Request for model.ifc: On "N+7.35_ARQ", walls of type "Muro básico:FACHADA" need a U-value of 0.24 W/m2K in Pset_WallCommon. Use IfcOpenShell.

First a look at what the model holds.

```python
import ifcopenshell
import ifcopenshell.util.element

model = ifcopenshell.open("model.ifc")
print(model.schema)
storey = next(s for s in model.by_type("IfcBuildingStorey") if s.Name == "N+7.35_ARQ")
walls = [e for e in ifcopenshell.util.element.get_decomposition(storey) if e.is_a("IfcWall")]
seen = {}
for e in walls:
    element_type = ifcopenshell.util.element.get_type(e)
    key = (element_type.Name if element_type != e and element_type else None, ifcopenshell.util.element.get_pset(e, "Pset_WallCommon", "ThermalTransmittance"))
    seen[key] = seen.get(key, 0) + 1
for (name, value), count in sorted(seen.items(), key=str):
    print(count, "x", name, "|", value)
```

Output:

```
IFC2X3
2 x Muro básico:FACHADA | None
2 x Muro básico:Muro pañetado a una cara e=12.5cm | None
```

```python
import ifcopenshell
import ifcopenshell.api.pset
import ifcopenshell.util.element

model = ifcopenshell.open("model.ifc")

storey = next(s for s in model.by_type("IfcBuildingStorey") if s.Name == "N+7.35_ARQ")
walls = [e for e in ifcopenshell.util.element.get_decomposition(storey) if e.is_a("IfcWall")]

count = 0
for e in walls:
    element_type = ifcopenshell.util.element.get_type(e)
    if element_type in (None, e) or element_type.Name != "Muro básico:FACHADA":
        continue
    # add_pset returns the element's existing set when there is one.
    pset = ifcopenshell.api.pset.add_pset(model, product=e, name="Pset_WallCommon")
    ifcopenshell.api.pset.edit_pset(model, pset=pset, properties={"ThermalTransmittance": 0.24})
    count += 1

print(count, "walls updated")

model.write("model_rev.ifc")
```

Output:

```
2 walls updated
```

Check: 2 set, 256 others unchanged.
